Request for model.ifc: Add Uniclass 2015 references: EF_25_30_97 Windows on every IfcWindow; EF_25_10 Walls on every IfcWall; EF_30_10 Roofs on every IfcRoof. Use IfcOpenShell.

First a look at what the model holds.

```python
import ifcopenshell

model = ifcopenshell.open("model.ifc")
print(model.schema)
print("classifications:", [c.Name for c in model.by_type("IfcClassification")])
for ifc_class in ("IfcDoor", "IfcRoof", "IfcStair", "IfcWall", "IfcWindow"):
    print(ifc_class, len(model.by_type(ifc_class)))
```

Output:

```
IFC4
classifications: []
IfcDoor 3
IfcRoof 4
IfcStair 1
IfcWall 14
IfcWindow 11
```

```python
import ifcopenshell
import ifcopenshell.api.classification

model = ifcopenshell.open("model.ifc")

system = ifcopenshell.api.classification.add_classification(model, classification="Uniclass 2015")

codes = {
    "IfcWindow": ("EF_25_30_97", "Windows"),
    "IfcWall": ("EF_25_10", "Walls"),
    "IfcRoof": ("EF_30_10", "Roofs"),
}
for ifc_class, (code, name) in codes.items():
    products = model.by_type(ifc_class)
    ifcopenshell.api.classification.add_reference(
        model, products=products, classification=system, identification=code, name=name
    )
    print(code, len(products))

model.write("model_rev.ifc")
```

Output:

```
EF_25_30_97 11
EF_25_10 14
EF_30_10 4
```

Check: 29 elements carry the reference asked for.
